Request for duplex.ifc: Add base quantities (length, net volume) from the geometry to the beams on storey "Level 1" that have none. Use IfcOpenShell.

First a look at what the model holds.

```python
import ifcopenshell
import ifcopenshell.util.element
import ifcopenshell.util.unit

model = ifcopenshell.open("duplex.ifc")
print(model.schema)
for unit_type in ("LENGTHUNIT", "AREAUNIT", "VOLUMEUNIT"):
    print(unit_type, ifcopenshell.util.unit.calculate_unit_scale(model, unit_type))
storey = next(s for s in model.by_type("IfcBuildingStorey") if s.Name == "Level 1")
beams = [e for e in ifcopenshell.util.element.get_decomposition(storey) if e.is_a("IfcBeam")]
for e in sorted(beams, key=lambda e: e.id()):
    print(e.id(), e.is_a(), e.Name, list(ifcopenshell.util.element.get_psets(e, qtos_only=True)), sep=" | ")
```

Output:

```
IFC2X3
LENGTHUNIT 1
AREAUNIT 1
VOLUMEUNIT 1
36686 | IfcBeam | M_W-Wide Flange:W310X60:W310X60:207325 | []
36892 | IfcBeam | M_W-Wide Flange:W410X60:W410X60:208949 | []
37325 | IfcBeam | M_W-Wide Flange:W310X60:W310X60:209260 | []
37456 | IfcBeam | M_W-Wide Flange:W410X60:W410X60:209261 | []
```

```python
import ifcopenshell
import ifcopenshell.api.pset
import ifcopenshell.geom
import ifcopenshell.util.element
import ifcopenshell.util.shape
import ifcopenshell.util.unit

model = ifcopenshell.open("duplex.ifc")
unit_scale = ifcopenshell.util.unit.calculate_unit_scale(model)
volume_scale = ifcopenshell.util.unit.calculate_unit_scale(model, "VOLUMEUNIT")
settings = ifcopenshell.geom.settings()

storey = next(s for s in model.by_type("IfcBuildingStorey") if s.Name == "Level 1")
beams = [e for e in ifcopenshell.util.element.get_decomposition(storey) if e.is_a("IfcBeam")]

for e in sorted(beams, key=lambda e: e.id()):
    if ifcopenshell.util.element.get_psets(e, qtos_only=True, should_inherit=False):
        continue
    # Geometry comes back in metres, in the element's own axes.
    shape = ifcopenshell.geom.create_shape(settings, e)
    values = {
        "Length": ifcopenshell.util.shape.get_max_xyz(shape.geometry) / unit_scale,
        "NetVolume": ifcopenshell.util.shape.get_volume(shape.geometry) / volume_scale,
    }
    qto = ifcopenshell.api.pset.add_qto(model, product=e, name="BaseQuantities")
    ifcopenshell.api.pset.edit_qto(model, qto=qto, properties=values)
    print(e.id(), {k: round(v, 3) for k, v in values.items()})

model.write("duplex_v2.ifc")
```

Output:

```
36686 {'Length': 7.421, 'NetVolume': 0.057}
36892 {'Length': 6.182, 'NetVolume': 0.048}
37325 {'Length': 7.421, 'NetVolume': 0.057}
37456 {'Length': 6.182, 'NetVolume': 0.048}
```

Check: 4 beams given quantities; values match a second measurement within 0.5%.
